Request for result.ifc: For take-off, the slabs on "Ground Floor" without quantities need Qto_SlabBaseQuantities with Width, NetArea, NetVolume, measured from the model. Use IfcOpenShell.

First a look at what the model holds.

```python
import ifcopenshell
import ifcopenshell.util.element
import ifcopenshell.util.unit

model = ifcopenshell.open("result.ifc")
print(model.schema)
for unit_type in ("LENGTHUNIT", "AREAUNIT", "VOLUMEUNIT"):
    print(unit_type, ifcopenshell.util.unit.calculate_unit_scale(model, unit_type))
storey = next(s for s in model.by_type("IfcBuildingStorey") if s.Name == "Ground Floor")
slabs = [e for e in ifcopenshell.util.element.get_decomposition(storey) if e.is_a("IfcSlab")]
for e in sorted(slabs, key=lambda e: e.id()):
    print(e.id(), e.is_a(), e.Name, list(ifcopenshell.util.element.get_psets(e, qtos_only=True)), sep=" | ")
```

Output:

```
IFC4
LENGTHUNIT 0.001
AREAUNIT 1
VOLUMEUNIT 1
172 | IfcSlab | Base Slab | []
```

```python
import ifcopenshell
import ifcopenshell.api.pset
import ifcopenshell.geom
import ifcopenshell.util.element
import ifcopenshell.util.shape
import ifcopenshell.util.unit

model = ifcopenshell.open("result.ifc")
unit_scale = ifcopenshell.util.unit.calculate_unit_scale(model)
area_scale = ifcopenshell.util.unit.calculate_unit_scale(model, "AREAUNIT")
volume_scale = ifcopenshell.util.unit.calculate_unit_scale(model, "VOLUMEUNIT")
settings = ifcopenshell.geom.settings()

storey = next(s for s in model.by_type("IfcBuildingStorey") if s.Name == "Ground Floor")
slabs = [e for e in ifcopenshell.util.element.get_decomposition(storey) if e.is_a("IfcSlab")]

for e in sorted(slabs, key=lambda e: e.id()):
    if ifcopenshell.util.element.get_psets(e, qtos_only=True, should_inherit=False):
        continue
    # Geometry comes back in metres, in the element's own axes.
    shape = ifcopenshell.geom.create_shape(settings, e)
    values = {
        "Width": ifcopenshell.util.shape.get_z(shape.geometry) / unit_scale,
        "NetArea": ifcopenshell.util.shape.get_footprint_area(shape.geometry) / area_scale,
        "NetVolume": ifcopenshell.util.shape.get_volume(shape.geometry) / volume_scale,
    }
    qto = ifcopenshell.api.pset.add_qto(model, product=e, name="Qto_SlabBaseQuantities")
    ifcopenshell.api.pset.edit_qto(model, qto=qto, properties=values)
    print(e.id(), {k: round(v, 3) for k, v in values.items()})

model.write("result_v2.ifc")
```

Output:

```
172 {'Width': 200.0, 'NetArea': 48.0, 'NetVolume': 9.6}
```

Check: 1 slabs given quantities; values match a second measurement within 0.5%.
